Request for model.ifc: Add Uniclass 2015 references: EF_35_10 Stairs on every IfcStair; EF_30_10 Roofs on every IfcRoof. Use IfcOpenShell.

First a look at what the model holds.

```python
import ifcopenshell

model = ifcopenshell.open("model.ifc")
print(model.schema)
print("classifications:", [c.Name for c in model.by_type("IfcClassification")])
for ifc_class in ("IfcDoor", "IfcRoof", "IfcStair", "IfcWall", "IfcWindow"):
    print(ifc_class, len(model.by_type(ifc_class)))
```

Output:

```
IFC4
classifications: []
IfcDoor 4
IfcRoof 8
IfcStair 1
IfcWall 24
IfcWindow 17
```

```python
import ifcopenshell
import ifcopenshell.api.classification

model = ifcopenshell.open("model.ifc")

system = ifcopenshell.api.classification.add_classification(model, classification="Uniclass 2015")

codes = {
    "IfcStair": ("EF_35_10", "Stairs"),
    "IfcRoof": ("EF_30_10", "Roofs"),
}
for ifc_class, (code, name) in codes.items():
    products = model.by_type(ifc_class)
    ifcopenshell.api.classification.add_reference(
        model, products=products, classification=system, identification=code, name=name
    )
    print(code, len(products))

model.write("model_edited.ifc")
```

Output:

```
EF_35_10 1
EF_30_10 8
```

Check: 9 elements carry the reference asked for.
